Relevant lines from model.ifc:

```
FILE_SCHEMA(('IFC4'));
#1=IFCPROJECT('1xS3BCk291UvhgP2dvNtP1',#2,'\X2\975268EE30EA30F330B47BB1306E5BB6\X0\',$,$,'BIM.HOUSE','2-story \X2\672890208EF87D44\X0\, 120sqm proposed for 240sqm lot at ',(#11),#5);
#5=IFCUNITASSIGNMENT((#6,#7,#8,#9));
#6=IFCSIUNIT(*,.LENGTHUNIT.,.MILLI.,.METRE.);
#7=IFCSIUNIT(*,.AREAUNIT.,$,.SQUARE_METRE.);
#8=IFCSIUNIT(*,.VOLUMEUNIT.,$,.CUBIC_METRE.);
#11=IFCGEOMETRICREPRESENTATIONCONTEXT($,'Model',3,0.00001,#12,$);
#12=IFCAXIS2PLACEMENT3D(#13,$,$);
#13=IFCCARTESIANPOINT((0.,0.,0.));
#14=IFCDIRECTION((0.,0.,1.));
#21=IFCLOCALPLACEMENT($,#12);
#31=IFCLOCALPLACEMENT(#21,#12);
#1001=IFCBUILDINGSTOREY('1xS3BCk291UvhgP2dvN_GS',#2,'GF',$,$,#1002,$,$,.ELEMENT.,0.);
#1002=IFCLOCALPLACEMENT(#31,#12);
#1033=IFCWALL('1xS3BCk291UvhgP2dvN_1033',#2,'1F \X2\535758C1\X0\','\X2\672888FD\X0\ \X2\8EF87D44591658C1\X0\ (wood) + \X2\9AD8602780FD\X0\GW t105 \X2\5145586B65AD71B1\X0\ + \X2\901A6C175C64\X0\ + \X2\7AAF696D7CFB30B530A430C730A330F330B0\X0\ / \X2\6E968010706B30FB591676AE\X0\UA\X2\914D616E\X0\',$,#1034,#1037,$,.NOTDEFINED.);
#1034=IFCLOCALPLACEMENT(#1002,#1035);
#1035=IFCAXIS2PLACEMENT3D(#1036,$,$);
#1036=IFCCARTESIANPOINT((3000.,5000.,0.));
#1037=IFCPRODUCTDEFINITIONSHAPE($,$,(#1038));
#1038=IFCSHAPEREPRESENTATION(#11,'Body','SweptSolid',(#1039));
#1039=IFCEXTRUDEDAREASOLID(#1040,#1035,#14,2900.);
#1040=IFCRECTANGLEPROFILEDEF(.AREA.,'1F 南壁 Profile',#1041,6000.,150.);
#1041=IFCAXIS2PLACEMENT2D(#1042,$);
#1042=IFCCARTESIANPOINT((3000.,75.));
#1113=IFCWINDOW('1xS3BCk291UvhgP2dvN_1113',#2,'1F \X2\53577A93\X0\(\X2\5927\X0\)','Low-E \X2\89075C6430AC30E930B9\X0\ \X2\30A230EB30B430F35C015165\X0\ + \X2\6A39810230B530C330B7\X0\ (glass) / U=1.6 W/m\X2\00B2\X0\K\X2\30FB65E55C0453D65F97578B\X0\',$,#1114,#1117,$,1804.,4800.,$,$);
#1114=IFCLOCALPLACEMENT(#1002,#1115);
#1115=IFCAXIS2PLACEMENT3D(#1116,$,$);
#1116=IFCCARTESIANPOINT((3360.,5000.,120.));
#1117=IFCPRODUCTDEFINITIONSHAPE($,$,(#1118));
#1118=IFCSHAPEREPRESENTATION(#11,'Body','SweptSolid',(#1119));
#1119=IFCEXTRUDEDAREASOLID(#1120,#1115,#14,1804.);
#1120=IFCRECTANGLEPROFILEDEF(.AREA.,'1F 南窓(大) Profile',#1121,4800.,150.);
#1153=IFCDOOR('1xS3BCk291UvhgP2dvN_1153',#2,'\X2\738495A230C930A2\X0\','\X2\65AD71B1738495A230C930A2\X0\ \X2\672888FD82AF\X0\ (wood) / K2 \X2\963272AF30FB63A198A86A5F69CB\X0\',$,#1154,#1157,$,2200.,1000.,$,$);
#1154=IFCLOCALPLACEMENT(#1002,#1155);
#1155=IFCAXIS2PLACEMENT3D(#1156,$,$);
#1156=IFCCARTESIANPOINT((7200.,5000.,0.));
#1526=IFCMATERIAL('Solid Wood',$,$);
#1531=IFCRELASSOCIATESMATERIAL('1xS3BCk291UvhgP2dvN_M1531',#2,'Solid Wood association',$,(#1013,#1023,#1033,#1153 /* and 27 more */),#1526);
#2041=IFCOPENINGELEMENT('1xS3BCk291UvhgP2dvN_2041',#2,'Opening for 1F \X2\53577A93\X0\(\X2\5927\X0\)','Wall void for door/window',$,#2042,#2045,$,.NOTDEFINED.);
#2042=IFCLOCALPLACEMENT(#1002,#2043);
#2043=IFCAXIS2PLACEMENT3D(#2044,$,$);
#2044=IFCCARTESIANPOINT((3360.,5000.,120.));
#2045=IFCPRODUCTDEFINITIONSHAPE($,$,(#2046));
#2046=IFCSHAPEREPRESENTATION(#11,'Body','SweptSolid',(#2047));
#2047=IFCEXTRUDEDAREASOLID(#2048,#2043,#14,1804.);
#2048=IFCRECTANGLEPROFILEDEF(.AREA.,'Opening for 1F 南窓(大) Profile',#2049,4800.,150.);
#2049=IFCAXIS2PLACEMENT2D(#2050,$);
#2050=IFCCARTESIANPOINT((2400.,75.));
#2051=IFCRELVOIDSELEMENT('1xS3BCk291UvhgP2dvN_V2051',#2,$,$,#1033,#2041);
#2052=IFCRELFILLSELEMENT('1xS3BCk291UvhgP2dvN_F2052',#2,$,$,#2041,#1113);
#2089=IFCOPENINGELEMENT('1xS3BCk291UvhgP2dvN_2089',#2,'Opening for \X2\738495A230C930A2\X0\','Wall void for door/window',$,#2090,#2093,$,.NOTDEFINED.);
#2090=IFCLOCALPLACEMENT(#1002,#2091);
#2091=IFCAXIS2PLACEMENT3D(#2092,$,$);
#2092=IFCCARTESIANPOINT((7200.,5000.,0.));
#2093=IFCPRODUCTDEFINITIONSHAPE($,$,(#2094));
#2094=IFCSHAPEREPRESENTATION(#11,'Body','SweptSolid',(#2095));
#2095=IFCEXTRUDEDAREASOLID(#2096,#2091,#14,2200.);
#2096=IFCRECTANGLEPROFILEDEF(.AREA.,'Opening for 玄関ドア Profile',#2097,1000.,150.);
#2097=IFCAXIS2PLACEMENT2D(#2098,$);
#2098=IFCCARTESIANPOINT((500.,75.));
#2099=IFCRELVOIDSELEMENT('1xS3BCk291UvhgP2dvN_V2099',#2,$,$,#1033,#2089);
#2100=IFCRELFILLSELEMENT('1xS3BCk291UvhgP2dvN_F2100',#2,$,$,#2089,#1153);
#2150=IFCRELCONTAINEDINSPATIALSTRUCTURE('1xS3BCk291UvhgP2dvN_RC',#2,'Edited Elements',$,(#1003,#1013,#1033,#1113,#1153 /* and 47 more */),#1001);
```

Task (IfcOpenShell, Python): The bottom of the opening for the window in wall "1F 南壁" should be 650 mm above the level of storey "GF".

```python
import numpy as np
import ifcopenshell
import ifcopenshell.api.geometry
import ifcopenshell.geom
import ifcopenshell.util.element
import ifcopenshell.util.placement
import ifcopenshell.util.shape
import ifcopenshell.util.unit

model = ifcopenshell.open("model.ifc")
unit_scale = ifcopenshell.util.unit.calculate_unit_scale(model)

window = model.by_id(1113)
opening = window.FillsVoids[0].RelatingOpeningElement
storey = ifcopenshell.util.element.get_container(window, ifc_class="IfcBuildingStorey")
level = ifcopenshell.util.placement.get_local_placement(storey.ObjectPlacement)[2, 3]

# The opening's origin need not be at the sill, so measure its lowest point.
shape = ifcopenshell.geom.create_shape(ifcopenshell.geom.settings(), opening)
bottom = ifcopenshell.util.shape.get_shape_bottom_elevation(shape, shape.geometry) / unit_scale
dz = level + 650.0 - bottom

shift = np.array([0.0, 0.0, dz])
# The window is not placed relative to its opening, so move both.
for product in (opening, window):
    matrix = ifcopenshell.util.placement.get_local_placement(product.ObjectPlacement)
    matrix[:3, 3] += shift
    ifcopenshell.api.geometry.edit_object_placement(model, product=product, matrix=matrix, is_si=False)

print(f"moved by {dz * unit_scale:+.3f} m")

model.write("model_updated.ifc")
```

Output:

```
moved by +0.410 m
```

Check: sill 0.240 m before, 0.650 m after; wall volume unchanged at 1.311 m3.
